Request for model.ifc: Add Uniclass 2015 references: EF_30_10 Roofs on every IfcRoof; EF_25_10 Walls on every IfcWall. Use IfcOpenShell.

First a look at what the model holds.

```python
import ifcopenshell

model = ifcopenshell.open("model.ifc")
print(model.schema)
print("classifications:", [c.Name for c in model.by_type("IfcClassification")])
for ifc_class in ("IfcDoor", "IfcRoof", "IfcStair", "IfcWall", "IfcWindow"):
    print(ifc_class, len(model.by_type(ifc_class)))
```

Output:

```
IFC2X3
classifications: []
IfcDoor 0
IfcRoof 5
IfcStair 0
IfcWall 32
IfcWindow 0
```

```python
import ifcopenshell
import ifcopenshell.api.classification

model = ifcopenshell.open("model.ifc")

# IFC2X3 requires Source and Edition and has no link from the project to the system.
system = model.create_entity("IfcClassification", Source="NBS", Edition="2015", Name="Uniclass 2015")

codes = {
    "IfcRoof": ("EF_30_10", "Roofs"),
    "IfcWall": ("EF_25_10", "Walls"),
}
for ifc_class, (code, name) in codes.items():
    products = model.by_type(ifc_class)
    ifcopenshell.api.classification.add_reference(
        model, products=products, classification=system, identification=code, name=name
    )
    print(code, len(products))

model.write("model_updated.ifc")
```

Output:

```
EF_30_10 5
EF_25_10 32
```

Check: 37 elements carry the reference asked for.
